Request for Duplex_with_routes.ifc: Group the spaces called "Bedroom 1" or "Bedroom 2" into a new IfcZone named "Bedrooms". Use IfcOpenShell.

First a look at what the model holds.

```python
import ifcopenshell

model = ifcopenshell.open("Duplex_with_routes.ifc")
print(model.schema)
seen = {}
for space in model.by_type("IfcSpace"):
    seen[space.LongName] = seen.get(space.LongName, 0) + 1
for name, count in sorted(seen.items(), key=str):
    print(count, "x", name)
print("zones:", [z.Name for z in model.by_type("IfcZone")][:20])
```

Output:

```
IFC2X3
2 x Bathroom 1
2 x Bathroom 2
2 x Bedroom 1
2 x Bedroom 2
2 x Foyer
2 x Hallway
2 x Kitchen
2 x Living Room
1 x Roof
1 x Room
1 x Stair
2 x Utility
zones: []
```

```python
import ifcopenshell
import ifcopenshell.api.group
import ifcopenshell.api.root

model = ifcopenshell.open("Duplex_with_routes.ifc")

names = {"Bedroom 1", "Bedroom 2"}
spaces = [s for s in model.by_type("IfcSpace") if s.LongName in names]

zone = ifcopenshell.api.root.create_entity(model, ifc_class="IfcZone", name="Bedrooms")
ifcopenshell.api.group.assign_group(model, products=spaces, group=zone)
print(len(spaces), "spaces in", zone.Name)

model.write("Duplex_with_routes_edited.ifc")
```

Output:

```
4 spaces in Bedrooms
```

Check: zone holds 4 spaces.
